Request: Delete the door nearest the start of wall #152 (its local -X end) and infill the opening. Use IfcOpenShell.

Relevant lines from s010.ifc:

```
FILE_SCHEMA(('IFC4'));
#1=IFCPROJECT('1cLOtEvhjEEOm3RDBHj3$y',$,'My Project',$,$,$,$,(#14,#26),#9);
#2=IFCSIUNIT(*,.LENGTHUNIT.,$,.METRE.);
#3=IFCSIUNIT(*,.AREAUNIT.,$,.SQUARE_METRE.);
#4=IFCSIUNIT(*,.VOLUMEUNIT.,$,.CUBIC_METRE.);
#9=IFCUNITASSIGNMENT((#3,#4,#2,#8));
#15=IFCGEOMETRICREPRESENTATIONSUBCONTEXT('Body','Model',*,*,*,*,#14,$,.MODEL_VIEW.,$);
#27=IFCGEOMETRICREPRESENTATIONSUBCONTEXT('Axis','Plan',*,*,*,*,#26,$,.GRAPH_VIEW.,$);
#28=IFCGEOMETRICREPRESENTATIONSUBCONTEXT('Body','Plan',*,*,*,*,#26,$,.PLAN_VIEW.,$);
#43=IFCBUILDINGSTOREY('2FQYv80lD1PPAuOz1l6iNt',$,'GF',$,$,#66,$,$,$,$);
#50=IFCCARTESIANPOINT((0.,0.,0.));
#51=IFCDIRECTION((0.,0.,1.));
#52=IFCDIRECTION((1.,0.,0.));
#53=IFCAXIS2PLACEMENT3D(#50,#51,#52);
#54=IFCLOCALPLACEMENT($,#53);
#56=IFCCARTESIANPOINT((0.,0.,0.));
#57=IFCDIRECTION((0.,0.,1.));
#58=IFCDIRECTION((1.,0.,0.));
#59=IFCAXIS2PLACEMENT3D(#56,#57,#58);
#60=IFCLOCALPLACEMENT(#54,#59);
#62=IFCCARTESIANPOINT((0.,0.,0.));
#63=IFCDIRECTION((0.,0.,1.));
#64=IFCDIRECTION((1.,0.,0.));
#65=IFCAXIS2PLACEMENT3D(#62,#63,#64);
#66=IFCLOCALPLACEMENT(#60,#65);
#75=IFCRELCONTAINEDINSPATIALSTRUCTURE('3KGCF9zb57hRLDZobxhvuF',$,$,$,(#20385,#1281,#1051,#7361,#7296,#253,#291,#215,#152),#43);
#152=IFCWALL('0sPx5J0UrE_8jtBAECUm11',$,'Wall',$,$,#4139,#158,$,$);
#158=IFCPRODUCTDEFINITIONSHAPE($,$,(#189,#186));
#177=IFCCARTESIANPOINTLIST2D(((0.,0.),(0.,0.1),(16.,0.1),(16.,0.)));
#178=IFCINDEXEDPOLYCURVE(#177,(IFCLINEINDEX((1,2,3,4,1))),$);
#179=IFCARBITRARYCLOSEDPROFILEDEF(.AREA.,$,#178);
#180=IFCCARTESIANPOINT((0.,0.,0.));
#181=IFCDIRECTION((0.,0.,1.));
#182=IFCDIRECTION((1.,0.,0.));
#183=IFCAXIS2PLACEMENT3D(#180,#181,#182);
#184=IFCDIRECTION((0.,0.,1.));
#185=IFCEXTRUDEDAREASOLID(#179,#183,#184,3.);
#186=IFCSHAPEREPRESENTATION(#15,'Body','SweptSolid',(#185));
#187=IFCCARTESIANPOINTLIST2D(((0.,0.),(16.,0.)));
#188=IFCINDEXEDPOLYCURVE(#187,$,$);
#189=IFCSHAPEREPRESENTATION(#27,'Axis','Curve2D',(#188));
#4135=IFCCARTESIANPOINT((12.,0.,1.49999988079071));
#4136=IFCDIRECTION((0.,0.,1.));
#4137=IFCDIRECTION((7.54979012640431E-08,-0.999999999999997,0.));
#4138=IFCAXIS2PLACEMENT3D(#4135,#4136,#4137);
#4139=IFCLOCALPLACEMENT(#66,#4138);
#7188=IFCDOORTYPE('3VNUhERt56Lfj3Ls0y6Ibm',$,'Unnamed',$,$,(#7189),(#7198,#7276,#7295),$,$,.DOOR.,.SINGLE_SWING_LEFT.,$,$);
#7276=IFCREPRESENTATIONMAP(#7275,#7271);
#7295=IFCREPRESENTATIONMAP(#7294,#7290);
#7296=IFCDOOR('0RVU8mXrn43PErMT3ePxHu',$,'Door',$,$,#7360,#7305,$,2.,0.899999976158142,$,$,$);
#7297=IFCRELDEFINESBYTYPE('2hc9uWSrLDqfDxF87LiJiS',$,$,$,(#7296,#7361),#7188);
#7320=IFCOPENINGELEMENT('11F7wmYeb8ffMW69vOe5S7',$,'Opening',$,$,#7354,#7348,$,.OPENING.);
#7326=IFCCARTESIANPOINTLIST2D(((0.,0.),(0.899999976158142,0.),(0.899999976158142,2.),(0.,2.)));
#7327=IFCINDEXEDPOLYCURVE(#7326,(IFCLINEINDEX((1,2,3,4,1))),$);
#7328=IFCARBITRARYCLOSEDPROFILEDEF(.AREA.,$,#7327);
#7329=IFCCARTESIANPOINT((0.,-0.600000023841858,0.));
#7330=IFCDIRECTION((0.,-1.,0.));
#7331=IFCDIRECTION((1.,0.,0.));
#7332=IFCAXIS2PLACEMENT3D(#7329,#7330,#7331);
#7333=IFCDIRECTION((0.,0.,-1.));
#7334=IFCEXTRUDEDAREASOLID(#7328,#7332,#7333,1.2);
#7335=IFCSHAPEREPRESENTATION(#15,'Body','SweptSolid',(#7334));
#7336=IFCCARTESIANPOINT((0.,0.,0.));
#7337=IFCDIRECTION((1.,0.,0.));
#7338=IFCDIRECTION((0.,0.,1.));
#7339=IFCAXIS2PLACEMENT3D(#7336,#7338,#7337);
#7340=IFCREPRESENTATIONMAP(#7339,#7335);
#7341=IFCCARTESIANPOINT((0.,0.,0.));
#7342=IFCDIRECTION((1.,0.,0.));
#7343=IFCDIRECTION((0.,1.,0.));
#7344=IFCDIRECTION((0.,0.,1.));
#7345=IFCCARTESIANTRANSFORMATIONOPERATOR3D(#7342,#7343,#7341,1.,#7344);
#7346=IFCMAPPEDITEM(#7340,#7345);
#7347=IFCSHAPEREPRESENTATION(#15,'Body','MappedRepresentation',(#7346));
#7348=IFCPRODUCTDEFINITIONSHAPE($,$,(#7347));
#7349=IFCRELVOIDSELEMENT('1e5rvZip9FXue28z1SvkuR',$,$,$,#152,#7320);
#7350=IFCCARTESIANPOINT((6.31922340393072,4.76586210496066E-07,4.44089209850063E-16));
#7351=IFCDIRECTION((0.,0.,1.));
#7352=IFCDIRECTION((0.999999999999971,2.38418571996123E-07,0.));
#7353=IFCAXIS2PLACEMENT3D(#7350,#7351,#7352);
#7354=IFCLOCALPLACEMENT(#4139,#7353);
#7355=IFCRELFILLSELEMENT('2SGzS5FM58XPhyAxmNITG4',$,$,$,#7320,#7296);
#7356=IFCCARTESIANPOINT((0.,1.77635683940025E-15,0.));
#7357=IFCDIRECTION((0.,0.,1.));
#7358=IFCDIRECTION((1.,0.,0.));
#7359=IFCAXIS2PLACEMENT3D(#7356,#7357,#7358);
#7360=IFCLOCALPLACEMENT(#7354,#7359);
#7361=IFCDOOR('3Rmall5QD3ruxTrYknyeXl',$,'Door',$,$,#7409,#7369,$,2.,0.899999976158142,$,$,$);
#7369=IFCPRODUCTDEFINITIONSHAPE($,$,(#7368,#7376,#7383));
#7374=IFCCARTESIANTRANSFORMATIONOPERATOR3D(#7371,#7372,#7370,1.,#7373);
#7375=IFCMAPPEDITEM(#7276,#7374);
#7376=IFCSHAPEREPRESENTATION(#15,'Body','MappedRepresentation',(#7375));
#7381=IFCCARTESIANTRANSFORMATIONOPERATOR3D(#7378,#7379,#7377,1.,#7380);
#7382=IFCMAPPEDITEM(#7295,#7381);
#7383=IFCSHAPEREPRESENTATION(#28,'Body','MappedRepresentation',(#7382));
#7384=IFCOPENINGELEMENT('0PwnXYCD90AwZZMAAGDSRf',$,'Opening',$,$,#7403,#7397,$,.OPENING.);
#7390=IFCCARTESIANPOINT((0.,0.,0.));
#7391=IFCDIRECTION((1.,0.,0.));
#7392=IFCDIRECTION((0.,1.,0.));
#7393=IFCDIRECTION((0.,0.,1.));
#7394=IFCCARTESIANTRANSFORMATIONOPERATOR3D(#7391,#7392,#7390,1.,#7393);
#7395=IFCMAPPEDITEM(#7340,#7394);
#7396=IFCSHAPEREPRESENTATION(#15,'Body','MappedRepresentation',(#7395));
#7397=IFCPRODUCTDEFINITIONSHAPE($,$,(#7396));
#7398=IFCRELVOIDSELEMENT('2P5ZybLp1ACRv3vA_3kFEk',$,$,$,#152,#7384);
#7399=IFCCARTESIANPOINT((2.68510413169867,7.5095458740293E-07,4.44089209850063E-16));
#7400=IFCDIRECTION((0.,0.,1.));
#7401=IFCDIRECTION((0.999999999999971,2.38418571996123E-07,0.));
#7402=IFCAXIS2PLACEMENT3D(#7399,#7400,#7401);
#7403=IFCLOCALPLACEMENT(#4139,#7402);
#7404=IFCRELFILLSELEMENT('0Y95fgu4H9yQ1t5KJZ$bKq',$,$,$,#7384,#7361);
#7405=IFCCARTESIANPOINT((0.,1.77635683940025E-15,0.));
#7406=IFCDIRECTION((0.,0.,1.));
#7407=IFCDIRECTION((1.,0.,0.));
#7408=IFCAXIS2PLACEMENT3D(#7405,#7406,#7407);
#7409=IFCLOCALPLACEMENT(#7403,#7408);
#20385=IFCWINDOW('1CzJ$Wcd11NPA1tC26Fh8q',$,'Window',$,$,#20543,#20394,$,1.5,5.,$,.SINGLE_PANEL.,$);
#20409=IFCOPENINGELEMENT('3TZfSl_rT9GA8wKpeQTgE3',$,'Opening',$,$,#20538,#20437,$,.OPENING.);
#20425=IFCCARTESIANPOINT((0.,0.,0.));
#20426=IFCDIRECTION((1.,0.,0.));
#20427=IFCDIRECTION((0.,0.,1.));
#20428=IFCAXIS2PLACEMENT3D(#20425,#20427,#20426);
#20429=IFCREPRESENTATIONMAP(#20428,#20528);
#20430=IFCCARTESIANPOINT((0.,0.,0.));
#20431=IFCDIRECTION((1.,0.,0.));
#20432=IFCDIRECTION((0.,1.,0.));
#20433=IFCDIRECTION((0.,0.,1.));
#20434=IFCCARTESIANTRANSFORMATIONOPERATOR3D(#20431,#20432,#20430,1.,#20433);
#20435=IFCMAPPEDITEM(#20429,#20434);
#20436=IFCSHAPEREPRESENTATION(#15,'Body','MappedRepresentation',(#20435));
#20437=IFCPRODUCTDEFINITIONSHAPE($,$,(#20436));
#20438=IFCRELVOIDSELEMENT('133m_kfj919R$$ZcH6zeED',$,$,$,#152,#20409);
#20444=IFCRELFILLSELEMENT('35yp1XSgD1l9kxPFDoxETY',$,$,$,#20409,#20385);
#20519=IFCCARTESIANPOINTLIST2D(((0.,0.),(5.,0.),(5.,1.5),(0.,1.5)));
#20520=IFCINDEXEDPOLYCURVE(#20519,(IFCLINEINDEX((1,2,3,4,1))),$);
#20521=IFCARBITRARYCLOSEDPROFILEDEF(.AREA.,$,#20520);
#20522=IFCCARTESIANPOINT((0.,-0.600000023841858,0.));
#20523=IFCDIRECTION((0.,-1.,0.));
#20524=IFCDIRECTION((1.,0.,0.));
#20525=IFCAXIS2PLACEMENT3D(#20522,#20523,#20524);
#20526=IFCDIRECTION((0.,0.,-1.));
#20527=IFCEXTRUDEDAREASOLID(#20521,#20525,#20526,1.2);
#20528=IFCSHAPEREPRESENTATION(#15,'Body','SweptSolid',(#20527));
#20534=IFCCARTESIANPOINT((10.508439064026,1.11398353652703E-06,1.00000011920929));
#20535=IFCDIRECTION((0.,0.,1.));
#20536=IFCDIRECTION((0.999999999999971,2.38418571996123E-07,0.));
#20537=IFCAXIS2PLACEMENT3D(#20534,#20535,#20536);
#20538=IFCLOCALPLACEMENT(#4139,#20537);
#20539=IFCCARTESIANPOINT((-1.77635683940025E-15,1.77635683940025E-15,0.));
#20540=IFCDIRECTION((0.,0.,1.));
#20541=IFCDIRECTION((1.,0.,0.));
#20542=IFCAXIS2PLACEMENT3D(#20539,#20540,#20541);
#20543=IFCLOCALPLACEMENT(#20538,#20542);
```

```python
import ifcopenshell
import ifcopenshell.api.feature
import ifcopenshell.api.root
import ifcopenshell.geom
import ifcopenshell.util.shape

model = ifcopenshell.open("s010.ifc")
settings = ifcopenshell.geom.settings()


def volume(element):
    """Net volume in cubic metres, openings subtracted."""
    shape = ifcopenshell.geom.create_shape(settings, element)
    return ifcopenshell.util.shape.get_volume(shape.geometry)


door = model.by_guid("3Rmall5QD3ruxTrYknyeXl")
opening = door.FillsVoids[0].RelatingOpeningElement
wall = opening.VoidsElements[0].RelatingBuildingElement
before = volume(wall)

ifcopenshell.api.root.remove_product(model, product=door)
ifcopenshell.api.feature.remove_feature(model, feature=opening)

after = volume(wall)

print(f"wall volume {before:.3f} -> {after:.3f} m3")

model.write("s010_updated.ifc")
```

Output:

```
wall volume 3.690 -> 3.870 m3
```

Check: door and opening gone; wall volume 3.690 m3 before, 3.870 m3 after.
